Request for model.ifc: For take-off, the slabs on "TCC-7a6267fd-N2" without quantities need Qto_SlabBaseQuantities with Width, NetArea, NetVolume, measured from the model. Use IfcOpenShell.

First a look at what the model holds.

```python
import ifcopenshell
import ifcopenshell.util.element
import ifcopenshell.util.unit

model = ifcopenshell.open("model.ifc")
print(model.schema)
for unit_type in ("LENGTHUNIT", "AREAUNIT", "VOLUMEUNIT"):
    print(unit_type, ifcopenshell.util.unit.calculate_unit_scale(model, unit_type))
storey = next(s for s in model.by_type("IfcBuildingStorey") if s.Name == "TCC-7a6267fd-N2")
slabs = [e for e in ifcopenshell.util.element.get_decomposition(storey) if e.is_a("IfcSlab")]
for e in sorted(slabs, key=lambda e: e.id()):
    print(e.id(), e.is_a(), e.Name, list(ifcopenshell.util.element.get_psets(e, qtos_only=True)), sep=" | ")
```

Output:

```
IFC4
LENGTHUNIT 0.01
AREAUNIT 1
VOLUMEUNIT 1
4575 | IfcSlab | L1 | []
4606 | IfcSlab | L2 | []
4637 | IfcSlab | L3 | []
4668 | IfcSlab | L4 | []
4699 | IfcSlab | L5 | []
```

```python
import ifcopenshell
import ifcopenshell.api.pset
import ifcopenshell.geom
import ifcopenshell.util.element
import ifcopenshell.util.shape
import ifcopenshell.util.unit

model = ifcopenshell.open("model.ifc")
unit_scale = ifcopenshell.util.unit.calculate_unit_scale(model)
area_scale = ifcopenshell.util.unit.calculate_unit_scale(model, "AREAUNIT")
volume_scale = ifcopenshell.util.unit.calculate_unit_scale(model, "VOLUMEUNIT")
settings = ifcopenshell.geom.settings()

storey = next(s for s in model.by_type("IfcBuildingStorey") if s.Name == "TCC-7a6267fd-N2")
slabs = [e for e in ifcopenshell.util.element.get_decomposition(storey) if e.is_a("IfcSlab")]

for e in sorted(slabs, key=lambda e: e.id()):
    if ifcopenshell.util.element.get_psets(e, qtos_only=True, should_inherit=False):
        continue
    # Geometry comes back in metres, in the element's own axes.
    shape = ifcopenshell.geom.create_shape(settings, e)
    values = {
        "Width": ifcopenshell.util.shape.get_z(shape.geometry) / unit_scale,
        "NetArea": ifcopenshell.util.shape.get_footprint_area(shape.geometry) / area_scale,
        "NetVolume": ifcopenshell.util.shape.get_volume(shape.geometry) / volume_scale,
    }
    qto = ifcopenshell.api.pset.add_qto(model, product=e, name="Qto_SlabBaseQuantities")
    ifcopenshell.api.pset.edit_qto(model, qto=qto, properties=values)
    print(e.id(), {k: round(v, 3) for k, v in values.items()})

model.write("model_rev.ifc")
```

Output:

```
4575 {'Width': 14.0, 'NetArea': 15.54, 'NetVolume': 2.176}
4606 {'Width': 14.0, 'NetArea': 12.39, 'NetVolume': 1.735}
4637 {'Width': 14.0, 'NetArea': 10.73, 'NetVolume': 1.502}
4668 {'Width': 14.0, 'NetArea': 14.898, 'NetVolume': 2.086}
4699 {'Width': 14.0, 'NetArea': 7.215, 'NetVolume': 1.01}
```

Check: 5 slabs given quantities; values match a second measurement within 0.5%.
